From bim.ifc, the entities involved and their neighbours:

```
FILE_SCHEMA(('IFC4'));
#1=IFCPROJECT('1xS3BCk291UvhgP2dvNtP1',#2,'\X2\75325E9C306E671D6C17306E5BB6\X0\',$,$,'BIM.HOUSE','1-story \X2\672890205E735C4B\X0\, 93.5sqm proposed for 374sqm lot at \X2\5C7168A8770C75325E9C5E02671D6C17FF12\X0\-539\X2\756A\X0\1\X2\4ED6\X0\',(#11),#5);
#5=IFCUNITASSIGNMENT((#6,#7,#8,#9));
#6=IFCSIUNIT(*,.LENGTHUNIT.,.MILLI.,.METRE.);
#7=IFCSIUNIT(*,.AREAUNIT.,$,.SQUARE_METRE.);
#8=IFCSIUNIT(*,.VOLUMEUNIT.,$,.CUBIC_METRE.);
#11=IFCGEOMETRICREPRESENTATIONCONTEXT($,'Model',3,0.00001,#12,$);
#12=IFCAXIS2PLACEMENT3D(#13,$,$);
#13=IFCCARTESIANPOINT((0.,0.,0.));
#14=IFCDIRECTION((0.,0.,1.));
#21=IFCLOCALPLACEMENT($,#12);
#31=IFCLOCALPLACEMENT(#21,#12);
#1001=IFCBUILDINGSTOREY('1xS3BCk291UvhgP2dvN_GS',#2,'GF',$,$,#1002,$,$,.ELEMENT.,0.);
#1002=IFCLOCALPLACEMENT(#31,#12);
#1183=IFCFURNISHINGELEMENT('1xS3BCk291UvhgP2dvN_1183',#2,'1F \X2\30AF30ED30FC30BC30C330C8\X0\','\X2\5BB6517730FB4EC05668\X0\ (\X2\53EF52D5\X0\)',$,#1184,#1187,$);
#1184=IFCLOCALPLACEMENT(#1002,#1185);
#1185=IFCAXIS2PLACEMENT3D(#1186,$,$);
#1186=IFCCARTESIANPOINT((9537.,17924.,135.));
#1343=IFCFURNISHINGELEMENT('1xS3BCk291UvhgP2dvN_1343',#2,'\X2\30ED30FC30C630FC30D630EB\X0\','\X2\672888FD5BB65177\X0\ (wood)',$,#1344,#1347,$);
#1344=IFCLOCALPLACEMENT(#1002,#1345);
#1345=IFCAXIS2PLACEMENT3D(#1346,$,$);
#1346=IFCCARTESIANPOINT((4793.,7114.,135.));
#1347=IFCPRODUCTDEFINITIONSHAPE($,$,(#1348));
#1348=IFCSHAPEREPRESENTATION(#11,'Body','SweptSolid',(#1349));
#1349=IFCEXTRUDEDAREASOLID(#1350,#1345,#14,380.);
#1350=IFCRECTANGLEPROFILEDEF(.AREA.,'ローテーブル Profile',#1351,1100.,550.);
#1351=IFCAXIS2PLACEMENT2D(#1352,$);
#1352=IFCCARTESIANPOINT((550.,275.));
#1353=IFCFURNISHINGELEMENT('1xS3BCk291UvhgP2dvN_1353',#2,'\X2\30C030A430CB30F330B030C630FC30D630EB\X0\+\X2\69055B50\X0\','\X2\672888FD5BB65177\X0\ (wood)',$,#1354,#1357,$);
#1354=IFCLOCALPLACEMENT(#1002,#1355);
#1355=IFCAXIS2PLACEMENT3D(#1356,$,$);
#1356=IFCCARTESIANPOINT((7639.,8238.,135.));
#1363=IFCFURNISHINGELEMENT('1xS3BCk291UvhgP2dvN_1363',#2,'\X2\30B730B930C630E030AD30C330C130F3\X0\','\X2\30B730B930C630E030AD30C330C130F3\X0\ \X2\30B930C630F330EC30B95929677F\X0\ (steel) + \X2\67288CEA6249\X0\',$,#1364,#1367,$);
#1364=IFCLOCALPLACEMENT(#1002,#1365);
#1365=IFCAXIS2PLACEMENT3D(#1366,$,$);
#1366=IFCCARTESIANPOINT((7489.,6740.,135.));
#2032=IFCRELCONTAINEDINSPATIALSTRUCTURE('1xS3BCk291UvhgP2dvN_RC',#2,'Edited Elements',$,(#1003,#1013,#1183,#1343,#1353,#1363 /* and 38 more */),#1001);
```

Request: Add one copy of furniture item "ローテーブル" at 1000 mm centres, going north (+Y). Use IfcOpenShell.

```python
import numpy as np
import ifcopenshell
import ifcopenshell.api.geometry
import ifcopenshell.api.root
import ifcopenshell.util.element
import ifcopenshell.util.placement

model = ifcopenshell.open("bim.ifc")


def reuse_history(source, copy):
    """copy_class also copies each property set's owner history, people and application; keep the originals."""
    for rel in copy.IsDefinedBy:
        if rel.is_a("IfcRelDefinesByProperties") and (history := rel.RelatingPropertyDefinition.OwnerHistory):
            rel.RelatingPropertyDefinition.OwnerHistory = source.OwnerHistory
            ifcopenshell.util.element.remove_deep2(model, history)


source = model.by_guid("1xS3BCk291UvhgP2dvN_1343")
base = ifcopenshell.util.placement.get_local_placement(source.ObjectPlacement)
step = np.array([0.0, 1.0, 0.0]) * 1000.0

for i in range(1, 2):
    copy = ifcopenshell.api.root.copy_class(model, product=source)
    copy.Representation = ifcopenshell.util.element.copy_deep(
        model, source.Representation, exclude=["IfcGeometricRepresentationContext", "IfcRepresentationMap"]
    )
    reuse_history(source, copy)
    matrix = base.copy()
    matrix[:3, 3] += i * step
    print("added at", matrix[:3, 3].round(3) + 0.0)
    ifcopenshell.api.geometry.edit_object_placement(model, product=copy, matrix=matrix, is_si=False)

model.write("bim_rev.ifc")
```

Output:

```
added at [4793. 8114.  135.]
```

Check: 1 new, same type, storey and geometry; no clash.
